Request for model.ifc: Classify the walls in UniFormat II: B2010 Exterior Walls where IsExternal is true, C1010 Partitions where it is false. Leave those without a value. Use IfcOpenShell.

First a look at what the model holds.

```python
import ifcopenshell
import ifcopenshell.util.element

model = ifcopenshell.open("model.ifc")
print(model.schema)
print("classifications:", [c.Name for c in model.by_type("IfcClassification")])
values = [ifcopenshell.util.element.get_pset(e, "Pset_WallCommon", "IsExternal") for e in model.by_type("IfcWall")]
for value in (True, False, None):
    print("IsExternal", value, values.count(value))
```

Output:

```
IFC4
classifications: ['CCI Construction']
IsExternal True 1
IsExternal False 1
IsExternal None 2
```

```python
import ifcopenshell
import ifcopenshell.api.classification
import ifcopenshell.util.element

model = ifcopenshell.open("model.ifc")

system = ifcopenshell.api.classification.add_classification(model, classification="UniFormat II")

walls = model.by_type("IfcWall")
external = {e: ifcopenshell.util.element.get_pset(e, "Pset_WallCommon", "IsExternal") for e in walls}
for flag, code, name in ((True, "B2010", "Exterior Walls"), (False, "C1010", "Partitions")):
    products = [e for e in walls if external[e] is flag]
    ifcopenshell.api.classification.add_reference(
        model, products=products, classification=system, identification=code, name=name
    )
    print(code, len(products))

model.write("model_v2.ifc")
```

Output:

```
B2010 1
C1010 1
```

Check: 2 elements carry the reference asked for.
